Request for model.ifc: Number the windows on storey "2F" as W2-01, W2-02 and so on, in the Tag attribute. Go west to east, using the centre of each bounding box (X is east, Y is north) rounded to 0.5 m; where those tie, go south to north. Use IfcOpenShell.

First a look at what the model holds.

```python
import ifcopenshell
import ifcopenshell.util.element
import ifcopenshell.util.placement

model = ifcopenshell.open("model.ifc")
print(model.schema)
storey = next(s for s in model.by_type("IfcBuildingStorey") if s.Name == "2F")
windows = [e for e in ifcopenshell.util.element.get_decomposition(storey) if e.is_a("IfcWindow")]
for e in sorted(windows, key=lambda e: e.id()):
    origin = ifcopenshell.util.placement.get_local_placement(e.ObjectPlacement)[:3, 3]
    print(e.id(), e.Tag, e.Name, origin.round(2) + 0.0, sep=" | ")
```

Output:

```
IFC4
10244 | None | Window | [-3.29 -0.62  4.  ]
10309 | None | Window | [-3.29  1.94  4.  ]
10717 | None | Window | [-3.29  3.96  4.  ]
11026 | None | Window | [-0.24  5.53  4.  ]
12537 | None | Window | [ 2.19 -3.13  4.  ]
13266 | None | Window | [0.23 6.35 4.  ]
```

```python
import ifcopenshell
import ifcopenshell.geom
import ifcopenshell.util.element
import ifcopenshell.util.shape

model = ifcopenshell.open("model.ifc")
settings = ifcopenshell.geom.settings()
settings.set("use-world-coords", True)


def centre(element):
    shape = ifcopenshell.geom.create_shape(settings, element)
    return ifcopenshell.util.shape.get_bbox_centroid(shape.geometry)


storey = next(s for s in model.by_type("IfcBuildingStorey") if s.Name == "2F")
windows = [e for e in ifcopenshell.util.element.get_decomposition(storey) if e.is_a("IfcWindow")]

# Insertion points can sit at a corner or the storey origin, so sort by the geometry (in metres).
centres = {e: centre(e) for e in windows}
windows.sort(key=lambda e: (round(centres[e][0] / 0.5), centres[e][1]))

for i, e in enumerate(windows, start=1):
    number = f"W2-{i:02d}"
    e.Tag = number
    print(e.id(), number)

model.write("model_v2.ifc")
```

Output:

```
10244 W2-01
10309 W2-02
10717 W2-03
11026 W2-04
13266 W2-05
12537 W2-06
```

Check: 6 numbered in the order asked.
